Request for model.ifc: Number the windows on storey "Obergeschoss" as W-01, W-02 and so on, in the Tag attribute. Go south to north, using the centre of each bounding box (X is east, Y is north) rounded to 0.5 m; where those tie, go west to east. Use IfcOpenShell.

First a look at what the model holds.

```python
import ifcopenshell
import ifcopenshell.util.element
import ifcopenshell.util.placement

model = ifcopenshell.open("model.ifc")
print(model.schema)
storey = next(s for s in model.by_type("IfcBuildingStorey") if s.Name == "Obergeschoss")
windows = [e for e in ifcopenshell.util.element.get_decomposition(storey) if e.is_a("IfcWindow")]
for e in sorted(windows, key=lambda e: e.id()):
    origin = ifcopenshell.util.placement.get_local_placement(e.ObjectPlacement)[:3, 3]
    print(e.id(), e.Tag, e.Name, origin.round(2) + 0.0, sep=" | ")
```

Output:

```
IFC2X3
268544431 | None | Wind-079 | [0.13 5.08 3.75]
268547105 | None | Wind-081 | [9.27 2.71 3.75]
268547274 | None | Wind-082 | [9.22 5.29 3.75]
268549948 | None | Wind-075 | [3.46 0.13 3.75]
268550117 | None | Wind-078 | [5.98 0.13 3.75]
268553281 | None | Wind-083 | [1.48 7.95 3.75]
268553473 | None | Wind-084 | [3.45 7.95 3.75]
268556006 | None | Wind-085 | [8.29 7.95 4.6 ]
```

```python
import ifcopenshell
import ifcopenshell.geom
import ifcopenshell.util.element
import ifcopenshell.util.shape

model = ifcopenshell.open("model.ifc")
settings = ifcopenshell.geom.settings()
settings.set("use-world-coords", True)


def centre(element):
    shape = ifcopenshell.geom.create_shape(settings, element)
    return ifcopenshell.util.shape.get_bbox_centroid(shape.geometry)


storey = next(s for s in model.by_type("IfcBuildingStorey") if s.Name == "Obergeschoss")
windows = [e for e in ifcopenshell.util.element.get_decomposition(storey) if e.is_a("IfcWindow")]

# Insertion points can sit at a corner or the storey origin, so sort by the geometry (in metres).
centres = {e: centre(e) for e in windows}
windows.sort(key=lambda e: (round(centres[e][1] / 0.5), centres[e][0]))

for i, e in enumerate(windows, start=1):
    number = f"W-{i:02d}"
    e.Tag = number
    print(e.id(), number)

model.write("model-out.ifc")
```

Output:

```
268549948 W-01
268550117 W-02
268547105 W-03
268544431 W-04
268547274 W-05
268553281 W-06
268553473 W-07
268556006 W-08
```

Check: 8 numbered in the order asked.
